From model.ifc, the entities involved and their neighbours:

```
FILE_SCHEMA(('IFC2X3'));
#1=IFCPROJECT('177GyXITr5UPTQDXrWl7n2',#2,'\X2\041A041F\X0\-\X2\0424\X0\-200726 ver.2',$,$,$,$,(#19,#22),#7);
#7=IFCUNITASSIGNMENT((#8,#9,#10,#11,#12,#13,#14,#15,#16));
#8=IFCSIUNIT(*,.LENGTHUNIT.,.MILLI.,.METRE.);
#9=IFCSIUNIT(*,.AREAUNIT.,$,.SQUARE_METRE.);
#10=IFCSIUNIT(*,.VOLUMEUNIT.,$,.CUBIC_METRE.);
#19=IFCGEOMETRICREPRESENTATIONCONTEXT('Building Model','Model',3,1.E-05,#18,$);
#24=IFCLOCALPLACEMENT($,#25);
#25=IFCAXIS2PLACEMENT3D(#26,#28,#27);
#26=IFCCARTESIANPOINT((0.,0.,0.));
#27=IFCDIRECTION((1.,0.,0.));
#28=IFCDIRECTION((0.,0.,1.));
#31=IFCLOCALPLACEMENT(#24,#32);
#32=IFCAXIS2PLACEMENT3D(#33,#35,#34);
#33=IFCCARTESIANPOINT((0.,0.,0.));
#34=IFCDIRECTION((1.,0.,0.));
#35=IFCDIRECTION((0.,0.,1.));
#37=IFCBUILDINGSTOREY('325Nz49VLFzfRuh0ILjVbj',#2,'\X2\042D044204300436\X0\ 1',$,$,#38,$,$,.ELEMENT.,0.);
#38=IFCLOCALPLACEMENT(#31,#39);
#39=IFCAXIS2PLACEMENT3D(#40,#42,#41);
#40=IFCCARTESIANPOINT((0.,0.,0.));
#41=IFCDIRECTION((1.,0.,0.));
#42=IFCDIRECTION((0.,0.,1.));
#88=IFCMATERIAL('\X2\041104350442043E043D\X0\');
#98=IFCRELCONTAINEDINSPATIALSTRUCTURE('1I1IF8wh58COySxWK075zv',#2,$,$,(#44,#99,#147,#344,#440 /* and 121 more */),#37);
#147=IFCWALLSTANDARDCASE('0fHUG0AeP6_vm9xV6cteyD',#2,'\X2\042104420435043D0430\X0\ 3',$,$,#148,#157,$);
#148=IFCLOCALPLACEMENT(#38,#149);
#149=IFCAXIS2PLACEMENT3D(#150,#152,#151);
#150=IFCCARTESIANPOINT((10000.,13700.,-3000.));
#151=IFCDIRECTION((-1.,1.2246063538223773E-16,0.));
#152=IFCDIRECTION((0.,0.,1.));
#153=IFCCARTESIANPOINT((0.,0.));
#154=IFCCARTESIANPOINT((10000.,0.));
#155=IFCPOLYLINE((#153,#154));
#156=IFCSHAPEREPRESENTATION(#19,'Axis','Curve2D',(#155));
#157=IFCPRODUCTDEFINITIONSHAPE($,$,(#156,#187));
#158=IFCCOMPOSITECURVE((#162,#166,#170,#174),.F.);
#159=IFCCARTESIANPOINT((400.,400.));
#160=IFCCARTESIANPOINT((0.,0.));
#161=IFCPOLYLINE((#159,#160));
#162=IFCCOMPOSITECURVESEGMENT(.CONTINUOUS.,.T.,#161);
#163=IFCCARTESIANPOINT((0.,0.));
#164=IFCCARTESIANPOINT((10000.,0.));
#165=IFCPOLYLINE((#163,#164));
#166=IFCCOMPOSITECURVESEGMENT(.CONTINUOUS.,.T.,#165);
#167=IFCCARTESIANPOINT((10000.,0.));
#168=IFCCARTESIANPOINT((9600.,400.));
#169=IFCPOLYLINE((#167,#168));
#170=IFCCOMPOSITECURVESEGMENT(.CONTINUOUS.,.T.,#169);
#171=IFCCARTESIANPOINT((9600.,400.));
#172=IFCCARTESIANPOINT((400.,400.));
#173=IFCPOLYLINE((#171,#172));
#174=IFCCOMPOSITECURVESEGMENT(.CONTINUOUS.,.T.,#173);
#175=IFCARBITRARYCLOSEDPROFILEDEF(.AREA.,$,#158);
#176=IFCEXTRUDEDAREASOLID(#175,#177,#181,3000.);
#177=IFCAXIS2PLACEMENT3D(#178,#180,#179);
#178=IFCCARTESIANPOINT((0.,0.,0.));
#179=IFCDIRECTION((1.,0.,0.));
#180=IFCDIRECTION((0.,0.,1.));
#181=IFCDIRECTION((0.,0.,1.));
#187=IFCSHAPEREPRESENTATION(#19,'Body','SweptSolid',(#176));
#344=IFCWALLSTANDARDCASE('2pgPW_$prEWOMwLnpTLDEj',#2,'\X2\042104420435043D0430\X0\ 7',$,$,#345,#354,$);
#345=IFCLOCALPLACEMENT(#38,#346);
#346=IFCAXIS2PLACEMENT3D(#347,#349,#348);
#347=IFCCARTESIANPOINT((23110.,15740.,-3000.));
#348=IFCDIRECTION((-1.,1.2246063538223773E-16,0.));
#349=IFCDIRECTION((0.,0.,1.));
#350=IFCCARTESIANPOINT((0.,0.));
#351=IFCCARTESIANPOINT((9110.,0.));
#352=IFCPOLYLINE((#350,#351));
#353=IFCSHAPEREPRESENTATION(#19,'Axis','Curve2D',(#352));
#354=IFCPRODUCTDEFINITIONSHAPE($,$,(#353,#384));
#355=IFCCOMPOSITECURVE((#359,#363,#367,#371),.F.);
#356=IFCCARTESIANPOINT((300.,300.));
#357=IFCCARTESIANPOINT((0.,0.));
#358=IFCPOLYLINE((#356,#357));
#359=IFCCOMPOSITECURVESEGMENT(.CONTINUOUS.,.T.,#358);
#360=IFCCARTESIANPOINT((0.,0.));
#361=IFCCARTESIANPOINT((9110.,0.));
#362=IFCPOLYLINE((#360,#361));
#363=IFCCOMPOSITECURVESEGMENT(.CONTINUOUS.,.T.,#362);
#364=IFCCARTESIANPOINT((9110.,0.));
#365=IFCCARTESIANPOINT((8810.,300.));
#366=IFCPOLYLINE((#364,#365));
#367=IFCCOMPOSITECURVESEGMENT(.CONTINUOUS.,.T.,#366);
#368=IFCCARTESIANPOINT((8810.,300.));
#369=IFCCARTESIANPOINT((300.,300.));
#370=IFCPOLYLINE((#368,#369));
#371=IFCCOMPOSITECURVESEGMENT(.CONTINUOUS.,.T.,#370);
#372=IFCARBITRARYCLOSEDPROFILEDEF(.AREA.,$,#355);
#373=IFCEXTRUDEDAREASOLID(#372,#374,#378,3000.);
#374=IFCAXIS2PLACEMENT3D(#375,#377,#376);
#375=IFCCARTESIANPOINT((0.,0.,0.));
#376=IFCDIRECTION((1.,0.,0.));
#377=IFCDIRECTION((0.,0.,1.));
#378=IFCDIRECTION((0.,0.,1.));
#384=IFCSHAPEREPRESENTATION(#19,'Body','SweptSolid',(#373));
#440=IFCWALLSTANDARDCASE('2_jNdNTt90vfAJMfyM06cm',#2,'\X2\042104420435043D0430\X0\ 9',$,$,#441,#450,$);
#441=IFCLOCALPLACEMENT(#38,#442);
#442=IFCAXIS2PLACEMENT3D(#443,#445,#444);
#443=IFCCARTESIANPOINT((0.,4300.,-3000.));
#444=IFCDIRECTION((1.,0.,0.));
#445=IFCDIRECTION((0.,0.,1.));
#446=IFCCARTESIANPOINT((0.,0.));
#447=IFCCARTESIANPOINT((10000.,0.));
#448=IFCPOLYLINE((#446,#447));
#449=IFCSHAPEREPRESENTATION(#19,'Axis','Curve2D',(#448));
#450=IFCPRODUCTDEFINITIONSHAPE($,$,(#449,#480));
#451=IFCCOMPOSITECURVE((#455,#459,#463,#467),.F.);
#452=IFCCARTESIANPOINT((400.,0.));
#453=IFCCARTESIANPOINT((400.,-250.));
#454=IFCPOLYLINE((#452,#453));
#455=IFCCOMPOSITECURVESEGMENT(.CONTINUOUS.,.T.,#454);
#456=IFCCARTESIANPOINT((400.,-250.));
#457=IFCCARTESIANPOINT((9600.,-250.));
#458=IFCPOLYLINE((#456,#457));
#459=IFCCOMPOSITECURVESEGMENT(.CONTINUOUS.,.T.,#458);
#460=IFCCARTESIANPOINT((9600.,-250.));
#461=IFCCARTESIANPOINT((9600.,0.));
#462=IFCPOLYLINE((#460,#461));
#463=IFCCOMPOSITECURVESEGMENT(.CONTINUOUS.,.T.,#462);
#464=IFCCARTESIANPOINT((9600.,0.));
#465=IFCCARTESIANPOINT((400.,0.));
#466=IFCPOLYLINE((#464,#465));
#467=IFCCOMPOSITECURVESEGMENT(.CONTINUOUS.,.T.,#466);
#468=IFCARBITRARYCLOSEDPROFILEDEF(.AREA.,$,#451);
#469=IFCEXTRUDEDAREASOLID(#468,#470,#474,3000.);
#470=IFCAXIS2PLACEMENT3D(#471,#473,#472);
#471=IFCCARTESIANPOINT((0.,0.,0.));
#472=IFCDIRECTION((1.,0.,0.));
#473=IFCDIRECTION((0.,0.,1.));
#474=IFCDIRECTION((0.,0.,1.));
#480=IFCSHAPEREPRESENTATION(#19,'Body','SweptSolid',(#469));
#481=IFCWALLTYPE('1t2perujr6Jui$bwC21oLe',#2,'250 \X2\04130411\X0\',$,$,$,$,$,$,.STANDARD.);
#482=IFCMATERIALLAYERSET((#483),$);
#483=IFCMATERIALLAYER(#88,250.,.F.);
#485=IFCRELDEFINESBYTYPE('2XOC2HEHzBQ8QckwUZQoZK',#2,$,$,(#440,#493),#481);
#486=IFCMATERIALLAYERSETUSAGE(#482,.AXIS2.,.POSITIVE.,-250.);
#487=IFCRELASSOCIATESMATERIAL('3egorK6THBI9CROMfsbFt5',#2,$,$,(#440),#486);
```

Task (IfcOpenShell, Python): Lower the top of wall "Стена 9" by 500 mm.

```python
import ifcopenshell
import ifcopenshell.geom
import ifcopenshell.util.shape
import ifcopenshell.util.unit

model = ifcopenshell.open("model.ifc")
unit_scale = ifcopenshell.util.unit.calculate_unit_scale(model)
settings = ifcopenshell.geom.settings()


def volume(element):
    """Net volume in cubic metres, openings subtracted."""
    shape = ifcopenshell.geom.create_shape(settings, element)
    return ifcopenshell.util.shape.get_volume(shape.geometry)


wall = model.by_guid("2_jNdNTt90vfAJMfyM06cm")
before = volume(wall)

body = next(r for r in wall.Representation.Representations if r.RepresentationIdentifier == "Body")
solid = body.Items[0]
old_height = solid.Depth
solid.Depth -= 0.5 / unit_scale
after = volume(wall)

print(f"height {old_height:g} -> {solid.Depth:g}, volume {before:.3f} -> {after:.3f} m3")

model.write("model_edited.ifc")
```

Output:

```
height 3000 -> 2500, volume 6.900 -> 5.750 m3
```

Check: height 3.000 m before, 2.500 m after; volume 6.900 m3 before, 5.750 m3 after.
